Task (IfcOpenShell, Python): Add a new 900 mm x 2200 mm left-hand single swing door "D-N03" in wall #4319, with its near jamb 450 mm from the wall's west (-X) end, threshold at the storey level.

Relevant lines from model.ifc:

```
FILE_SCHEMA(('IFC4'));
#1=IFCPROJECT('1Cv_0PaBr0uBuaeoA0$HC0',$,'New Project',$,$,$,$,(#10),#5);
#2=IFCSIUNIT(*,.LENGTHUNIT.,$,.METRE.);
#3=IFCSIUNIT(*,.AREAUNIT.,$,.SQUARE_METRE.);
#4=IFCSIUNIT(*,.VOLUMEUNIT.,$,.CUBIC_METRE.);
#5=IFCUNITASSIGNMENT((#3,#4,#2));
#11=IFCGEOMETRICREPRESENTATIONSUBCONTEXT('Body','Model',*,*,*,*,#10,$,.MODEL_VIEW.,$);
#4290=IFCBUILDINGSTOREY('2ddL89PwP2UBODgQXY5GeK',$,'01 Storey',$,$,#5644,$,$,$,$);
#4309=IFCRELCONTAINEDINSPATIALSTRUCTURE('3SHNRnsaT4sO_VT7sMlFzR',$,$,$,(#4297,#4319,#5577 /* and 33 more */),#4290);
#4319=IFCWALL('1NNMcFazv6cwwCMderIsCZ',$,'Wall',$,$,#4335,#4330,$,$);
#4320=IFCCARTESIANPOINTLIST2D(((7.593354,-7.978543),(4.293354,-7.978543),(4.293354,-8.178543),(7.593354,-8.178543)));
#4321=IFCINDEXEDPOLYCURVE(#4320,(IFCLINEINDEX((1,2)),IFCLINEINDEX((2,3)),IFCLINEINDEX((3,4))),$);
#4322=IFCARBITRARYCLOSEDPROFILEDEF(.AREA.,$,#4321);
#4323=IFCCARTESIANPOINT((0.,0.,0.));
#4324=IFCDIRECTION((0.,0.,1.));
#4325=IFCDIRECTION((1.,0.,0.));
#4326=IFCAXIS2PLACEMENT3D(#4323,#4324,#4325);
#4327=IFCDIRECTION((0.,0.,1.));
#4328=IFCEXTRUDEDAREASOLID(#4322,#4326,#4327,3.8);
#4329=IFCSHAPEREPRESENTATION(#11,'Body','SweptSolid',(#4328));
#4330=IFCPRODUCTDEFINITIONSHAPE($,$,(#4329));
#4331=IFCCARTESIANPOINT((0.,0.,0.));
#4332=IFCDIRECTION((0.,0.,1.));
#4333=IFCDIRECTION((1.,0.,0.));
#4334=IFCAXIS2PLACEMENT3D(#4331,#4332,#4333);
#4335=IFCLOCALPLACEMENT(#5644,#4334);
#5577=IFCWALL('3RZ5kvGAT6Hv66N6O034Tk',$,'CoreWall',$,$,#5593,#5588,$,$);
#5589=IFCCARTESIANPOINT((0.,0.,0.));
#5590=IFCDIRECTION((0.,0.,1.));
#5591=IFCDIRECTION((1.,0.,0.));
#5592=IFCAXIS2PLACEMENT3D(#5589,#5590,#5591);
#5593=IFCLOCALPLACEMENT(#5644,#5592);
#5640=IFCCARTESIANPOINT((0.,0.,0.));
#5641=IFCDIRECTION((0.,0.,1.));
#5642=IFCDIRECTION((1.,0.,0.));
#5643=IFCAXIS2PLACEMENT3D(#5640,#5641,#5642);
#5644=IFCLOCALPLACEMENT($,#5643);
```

```python
import numpy as np
import ifcopenshell
import ifcopenshell.api.feature
import ifcopenshell.api.geometry
import ifcopenshell.api.root
import ifcopenshell.api.spatial
import ifcopenshell.geom
import ifcopenshell.util.element
import ifcopenshell.util.placement
import ifcopenshell.util.representation
import ifcopenshell.util.shape
import ifcopenshell.util.unit

model = ifcopenshell.open("model.ifc")
unit_scale = ifcopenshell.util.unit.calculate_unit_scale(model)
settings = ifcopenshell.geom.settings()


def volume(element):
    """Net volume in cubic metres, openings subtracted."""
    shape = ifcopenshell.geom.create_shape(settings, element)
    return ifcopenshell.util.shape.get_volume(shape.geometry)


wall = model.by_guid("1NNMcFazv6cwwCMderIsCZ")
storey = ifcopenshell.util.element.get_container(wall, ifc_class="IfcBuildingStorey")
context = ifcopenshell.util.representation.get_context(model, "Model", "Body", "MODEL_VIEW")
before = volume(wall)

width, height, from_end, sill = 0.9, 2.2, 0.45, 0.0  # metres

# The wall runs along its own X axis, and the end named is its -X end.
wall_shape = ifcopenshell.geom.create_shape(settings, wall)
x, y, z = ifcopenshell.util.shape.get_vertices(wall_shape.geometry).T
start = x.min() + from_end
face, thickness = float(y.min()), float(y.max() - y.min())
wall_matrix = ifcopenshell.util.placement.get_local_placement(wall.ObjectPlacement)
level = ifcopenshell.util.placement.get_local_placement(storey.ObjectPlacement)[2, 3]


def in_wall(x, y):
    """Placement at x, y metres in the wall's axes, at sill height."""
    matrix = wall_matrix.copy()
    matrix[:, 3] = wall_matrix @ np.array([x / unit_scale, y / unit_scale, 0.0, 1.0])
    matrix[2, 3] = level + sill / unit_scale
    return matrix


# Opening: a box that overshoots both wall faces by 50 mm.
opening = ifcopenshell.api.root.create_entity(model, ifc_class="IfcOpeningElement", predefined_type="OPENING")
box = ifcopenshell.api.geometry.add_wall_representation(
    model, context=context, length=width, height=height, thickness=thickness + 0.1
)
ifcopenshell.api.geometry.assign_representation(model, product=opening, representation=box)
ifcopenshell.api.geometry.edit_object_placement(model, product=opening, matrix=in_wall(start, face - 0.05), is_si=False)
ifcopenshell.api.feature.add_feature(model, feature=opening, element=wall)

door = ifcopenshell.api.root.create_entity(model, ifc_class="IfcDoor", name="D-N03", predefined_type="DOOR")
door.OverallWidth, door.OverallHeight = width / unit_scale, height / unit_scale
door.OperationType = "SINGLE_SWING_LEFT"
body = ifcopenshell.api.geometry.add_door_representation(
    model,
    context=context,
    overall_width=door.OverallWidth,
    overall_height=door.OverallHeight,
    operation_type="SINGLE_SWING_LEFT",
    lining_properties={"LiningDepth": thickness / unit_scale, "ThresholdDepth": thickness / unit_scale},
)
ifcopenshell.api.geometry.assign_representation(model, product=door, representation=body)
ifcopenshell.api.spatial.assign_container(model, products=[door], relating_structure=storey)
ifcopenshell.api.feature.add_filling(model, opening=opening, element=door)

# The lining spans the wall, so the door starts at the wall face.
ifcopenshell.api.geometry.edit_object_placement(model, product=door, matrix=in_wall(start, face), is_si=False)

after = volume(wall)

print(f"wall volume {before:.3f} -> {after:.3f} m3")

model.write("model_rev.ifc")
```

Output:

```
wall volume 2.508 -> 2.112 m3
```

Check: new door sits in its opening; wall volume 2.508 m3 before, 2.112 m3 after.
